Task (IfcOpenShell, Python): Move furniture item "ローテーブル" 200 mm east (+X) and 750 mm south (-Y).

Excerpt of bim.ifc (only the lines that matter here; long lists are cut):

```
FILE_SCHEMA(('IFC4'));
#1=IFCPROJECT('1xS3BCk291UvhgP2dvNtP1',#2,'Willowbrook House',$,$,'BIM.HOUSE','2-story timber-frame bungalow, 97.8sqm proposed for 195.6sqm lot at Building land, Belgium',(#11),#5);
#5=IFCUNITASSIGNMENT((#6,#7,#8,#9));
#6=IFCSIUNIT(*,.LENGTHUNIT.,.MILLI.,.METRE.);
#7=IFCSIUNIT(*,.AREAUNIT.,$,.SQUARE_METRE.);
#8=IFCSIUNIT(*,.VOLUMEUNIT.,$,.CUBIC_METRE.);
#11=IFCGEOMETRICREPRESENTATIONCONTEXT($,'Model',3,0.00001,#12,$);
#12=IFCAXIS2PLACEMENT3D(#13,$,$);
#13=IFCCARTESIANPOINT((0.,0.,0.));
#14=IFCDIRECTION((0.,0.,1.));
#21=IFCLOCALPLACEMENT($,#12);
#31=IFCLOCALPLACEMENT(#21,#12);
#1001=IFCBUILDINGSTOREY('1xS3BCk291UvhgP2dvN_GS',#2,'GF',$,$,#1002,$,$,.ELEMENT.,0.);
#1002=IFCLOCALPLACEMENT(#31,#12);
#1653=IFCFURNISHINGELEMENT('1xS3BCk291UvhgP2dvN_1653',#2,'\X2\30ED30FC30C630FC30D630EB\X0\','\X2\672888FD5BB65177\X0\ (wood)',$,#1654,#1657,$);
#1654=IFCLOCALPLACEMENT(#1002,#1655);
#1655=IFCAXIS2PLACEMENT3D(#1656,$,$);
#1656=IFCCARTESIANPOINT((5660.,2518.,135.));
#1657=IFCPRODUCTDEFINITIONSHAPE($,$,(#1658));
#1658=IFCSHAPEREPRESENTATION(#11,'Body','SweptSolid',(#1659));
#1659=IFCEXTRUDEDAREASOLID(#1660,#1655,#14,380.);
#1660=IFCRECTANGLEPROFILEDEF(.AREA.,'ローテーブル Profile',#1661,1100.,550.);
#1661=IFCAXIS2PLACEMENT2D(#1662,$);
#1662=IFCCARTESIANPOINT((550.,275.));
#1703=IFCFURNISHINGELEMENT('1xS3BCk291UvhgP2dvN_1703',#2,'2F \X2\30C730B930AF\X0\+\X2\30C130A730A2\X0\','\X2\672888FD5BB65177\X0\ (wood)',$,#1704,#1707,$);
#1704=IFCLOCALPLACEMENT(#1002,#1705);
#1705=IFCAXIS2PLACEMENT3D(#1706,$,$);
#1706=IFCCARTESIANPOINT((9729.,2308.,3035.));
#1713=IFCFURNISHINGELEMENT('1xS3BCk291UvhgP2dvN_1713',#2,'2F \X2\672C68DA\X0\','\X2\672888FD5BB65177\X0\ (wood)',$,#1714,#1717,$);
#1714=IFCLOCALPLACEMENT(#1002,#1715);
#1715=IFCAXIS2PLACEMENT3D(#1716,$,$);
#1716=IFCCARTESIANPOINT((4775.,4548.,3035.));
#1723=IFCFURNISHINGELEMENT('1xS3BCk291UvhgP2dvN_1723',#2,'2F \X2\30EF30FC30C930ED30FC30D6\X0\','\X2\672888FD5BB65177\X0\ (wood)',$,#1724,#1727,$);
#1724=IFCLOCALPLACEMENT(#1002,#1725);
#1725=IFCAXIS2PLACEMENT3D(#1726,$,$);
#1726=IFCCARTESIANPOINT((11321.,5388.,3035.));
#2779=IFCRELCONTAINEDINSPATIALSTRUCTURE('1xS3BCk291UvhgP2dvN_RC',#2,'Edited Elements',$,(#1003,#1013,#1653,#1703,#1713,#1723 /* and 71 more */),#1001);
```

```python
import ifcopenshell
import ifcopenshell.api.geometry
import ifcopenshell.util.placement
import ifcopenshell.util.unit

model = ifcopenshell.open("bim.ifc")
unit_scale = ifcopenshell.util.unit.calculate_unit_scale(model)

item = model.by_id(1653)
matrix = ifcopenshell.util.placement.get_local_placement(item.ObjectPlacement)
matrix[0, 3] += 0.2 / unit_scale
matrix[1, 3] -= 0.75 / unit_scale
ifcopenshell.api.geometry.edit_object_placement(model, product=item, matrix=matrix, is_si=False)

print(ifcopenshell.util.placement.get_local_placement(item.ObjectPlacement).round(3) + 0.0)

model.write("bim_edited.ifc")
```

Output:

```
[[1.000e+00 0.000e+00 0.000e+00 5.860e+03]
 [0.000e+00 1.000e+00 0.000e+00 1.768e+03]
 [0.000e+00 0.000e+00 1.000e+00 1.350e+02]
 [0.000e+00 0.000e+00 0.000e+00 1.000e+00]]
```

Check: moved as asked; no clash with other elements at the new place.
